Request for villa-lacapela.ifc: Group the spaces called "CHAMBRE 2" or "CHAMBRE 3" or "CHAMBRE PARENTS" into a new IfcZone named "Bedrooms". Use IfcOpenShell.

First a look at what the model holds.

```python
import ifcopenshell

model = ifcopenshell.open("villa-lacapela.ifc")
print(model.schema)
seen = {}
for space in model.by_type("IfcSpace"):
    seen[space.LongName] = seen.get(space.LongName, 0) + 1
for name, count in sorted(seen.items(), key=str):
    print(count, "x", name)
print("zones:", [z.Name for z in model.by_type("IfcZone")][:20])
```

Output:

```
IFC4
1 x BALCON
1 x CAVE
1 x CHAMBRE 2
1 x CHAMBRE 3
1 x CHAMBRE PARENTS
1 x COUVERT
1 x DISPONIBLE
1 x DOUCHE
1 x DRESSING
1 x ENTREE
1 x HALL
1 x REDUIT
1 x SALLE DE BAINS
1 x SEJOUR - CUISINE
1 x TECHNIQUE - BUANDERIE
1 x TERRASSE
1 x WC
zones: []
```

```python
import ifcopenshell
import ifcopenshell.api.group
import ifcopenshell.api.root

model = ifcopenshell.open("villa-lacapela.ifc")

names = {"CHAMBRE 2", "CHAMBRE 3", "CHAMBRE PARENTS"}
spaces = [s for s in model.by_type("IfcSpace") if s.LongName in names]

zone = ifcopenshell.api.root.create_entity(model, ifc_class="IfcZone", name="Bedrooms")
ifcopenshell.api.group.assign_group(model, products=spaces, group=zone)
print(len(spaces), "spaces in", zone.Name)

model.write("villa-lacapela-out.ifc")
```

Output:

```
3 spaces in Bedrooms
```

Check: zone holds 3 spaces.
